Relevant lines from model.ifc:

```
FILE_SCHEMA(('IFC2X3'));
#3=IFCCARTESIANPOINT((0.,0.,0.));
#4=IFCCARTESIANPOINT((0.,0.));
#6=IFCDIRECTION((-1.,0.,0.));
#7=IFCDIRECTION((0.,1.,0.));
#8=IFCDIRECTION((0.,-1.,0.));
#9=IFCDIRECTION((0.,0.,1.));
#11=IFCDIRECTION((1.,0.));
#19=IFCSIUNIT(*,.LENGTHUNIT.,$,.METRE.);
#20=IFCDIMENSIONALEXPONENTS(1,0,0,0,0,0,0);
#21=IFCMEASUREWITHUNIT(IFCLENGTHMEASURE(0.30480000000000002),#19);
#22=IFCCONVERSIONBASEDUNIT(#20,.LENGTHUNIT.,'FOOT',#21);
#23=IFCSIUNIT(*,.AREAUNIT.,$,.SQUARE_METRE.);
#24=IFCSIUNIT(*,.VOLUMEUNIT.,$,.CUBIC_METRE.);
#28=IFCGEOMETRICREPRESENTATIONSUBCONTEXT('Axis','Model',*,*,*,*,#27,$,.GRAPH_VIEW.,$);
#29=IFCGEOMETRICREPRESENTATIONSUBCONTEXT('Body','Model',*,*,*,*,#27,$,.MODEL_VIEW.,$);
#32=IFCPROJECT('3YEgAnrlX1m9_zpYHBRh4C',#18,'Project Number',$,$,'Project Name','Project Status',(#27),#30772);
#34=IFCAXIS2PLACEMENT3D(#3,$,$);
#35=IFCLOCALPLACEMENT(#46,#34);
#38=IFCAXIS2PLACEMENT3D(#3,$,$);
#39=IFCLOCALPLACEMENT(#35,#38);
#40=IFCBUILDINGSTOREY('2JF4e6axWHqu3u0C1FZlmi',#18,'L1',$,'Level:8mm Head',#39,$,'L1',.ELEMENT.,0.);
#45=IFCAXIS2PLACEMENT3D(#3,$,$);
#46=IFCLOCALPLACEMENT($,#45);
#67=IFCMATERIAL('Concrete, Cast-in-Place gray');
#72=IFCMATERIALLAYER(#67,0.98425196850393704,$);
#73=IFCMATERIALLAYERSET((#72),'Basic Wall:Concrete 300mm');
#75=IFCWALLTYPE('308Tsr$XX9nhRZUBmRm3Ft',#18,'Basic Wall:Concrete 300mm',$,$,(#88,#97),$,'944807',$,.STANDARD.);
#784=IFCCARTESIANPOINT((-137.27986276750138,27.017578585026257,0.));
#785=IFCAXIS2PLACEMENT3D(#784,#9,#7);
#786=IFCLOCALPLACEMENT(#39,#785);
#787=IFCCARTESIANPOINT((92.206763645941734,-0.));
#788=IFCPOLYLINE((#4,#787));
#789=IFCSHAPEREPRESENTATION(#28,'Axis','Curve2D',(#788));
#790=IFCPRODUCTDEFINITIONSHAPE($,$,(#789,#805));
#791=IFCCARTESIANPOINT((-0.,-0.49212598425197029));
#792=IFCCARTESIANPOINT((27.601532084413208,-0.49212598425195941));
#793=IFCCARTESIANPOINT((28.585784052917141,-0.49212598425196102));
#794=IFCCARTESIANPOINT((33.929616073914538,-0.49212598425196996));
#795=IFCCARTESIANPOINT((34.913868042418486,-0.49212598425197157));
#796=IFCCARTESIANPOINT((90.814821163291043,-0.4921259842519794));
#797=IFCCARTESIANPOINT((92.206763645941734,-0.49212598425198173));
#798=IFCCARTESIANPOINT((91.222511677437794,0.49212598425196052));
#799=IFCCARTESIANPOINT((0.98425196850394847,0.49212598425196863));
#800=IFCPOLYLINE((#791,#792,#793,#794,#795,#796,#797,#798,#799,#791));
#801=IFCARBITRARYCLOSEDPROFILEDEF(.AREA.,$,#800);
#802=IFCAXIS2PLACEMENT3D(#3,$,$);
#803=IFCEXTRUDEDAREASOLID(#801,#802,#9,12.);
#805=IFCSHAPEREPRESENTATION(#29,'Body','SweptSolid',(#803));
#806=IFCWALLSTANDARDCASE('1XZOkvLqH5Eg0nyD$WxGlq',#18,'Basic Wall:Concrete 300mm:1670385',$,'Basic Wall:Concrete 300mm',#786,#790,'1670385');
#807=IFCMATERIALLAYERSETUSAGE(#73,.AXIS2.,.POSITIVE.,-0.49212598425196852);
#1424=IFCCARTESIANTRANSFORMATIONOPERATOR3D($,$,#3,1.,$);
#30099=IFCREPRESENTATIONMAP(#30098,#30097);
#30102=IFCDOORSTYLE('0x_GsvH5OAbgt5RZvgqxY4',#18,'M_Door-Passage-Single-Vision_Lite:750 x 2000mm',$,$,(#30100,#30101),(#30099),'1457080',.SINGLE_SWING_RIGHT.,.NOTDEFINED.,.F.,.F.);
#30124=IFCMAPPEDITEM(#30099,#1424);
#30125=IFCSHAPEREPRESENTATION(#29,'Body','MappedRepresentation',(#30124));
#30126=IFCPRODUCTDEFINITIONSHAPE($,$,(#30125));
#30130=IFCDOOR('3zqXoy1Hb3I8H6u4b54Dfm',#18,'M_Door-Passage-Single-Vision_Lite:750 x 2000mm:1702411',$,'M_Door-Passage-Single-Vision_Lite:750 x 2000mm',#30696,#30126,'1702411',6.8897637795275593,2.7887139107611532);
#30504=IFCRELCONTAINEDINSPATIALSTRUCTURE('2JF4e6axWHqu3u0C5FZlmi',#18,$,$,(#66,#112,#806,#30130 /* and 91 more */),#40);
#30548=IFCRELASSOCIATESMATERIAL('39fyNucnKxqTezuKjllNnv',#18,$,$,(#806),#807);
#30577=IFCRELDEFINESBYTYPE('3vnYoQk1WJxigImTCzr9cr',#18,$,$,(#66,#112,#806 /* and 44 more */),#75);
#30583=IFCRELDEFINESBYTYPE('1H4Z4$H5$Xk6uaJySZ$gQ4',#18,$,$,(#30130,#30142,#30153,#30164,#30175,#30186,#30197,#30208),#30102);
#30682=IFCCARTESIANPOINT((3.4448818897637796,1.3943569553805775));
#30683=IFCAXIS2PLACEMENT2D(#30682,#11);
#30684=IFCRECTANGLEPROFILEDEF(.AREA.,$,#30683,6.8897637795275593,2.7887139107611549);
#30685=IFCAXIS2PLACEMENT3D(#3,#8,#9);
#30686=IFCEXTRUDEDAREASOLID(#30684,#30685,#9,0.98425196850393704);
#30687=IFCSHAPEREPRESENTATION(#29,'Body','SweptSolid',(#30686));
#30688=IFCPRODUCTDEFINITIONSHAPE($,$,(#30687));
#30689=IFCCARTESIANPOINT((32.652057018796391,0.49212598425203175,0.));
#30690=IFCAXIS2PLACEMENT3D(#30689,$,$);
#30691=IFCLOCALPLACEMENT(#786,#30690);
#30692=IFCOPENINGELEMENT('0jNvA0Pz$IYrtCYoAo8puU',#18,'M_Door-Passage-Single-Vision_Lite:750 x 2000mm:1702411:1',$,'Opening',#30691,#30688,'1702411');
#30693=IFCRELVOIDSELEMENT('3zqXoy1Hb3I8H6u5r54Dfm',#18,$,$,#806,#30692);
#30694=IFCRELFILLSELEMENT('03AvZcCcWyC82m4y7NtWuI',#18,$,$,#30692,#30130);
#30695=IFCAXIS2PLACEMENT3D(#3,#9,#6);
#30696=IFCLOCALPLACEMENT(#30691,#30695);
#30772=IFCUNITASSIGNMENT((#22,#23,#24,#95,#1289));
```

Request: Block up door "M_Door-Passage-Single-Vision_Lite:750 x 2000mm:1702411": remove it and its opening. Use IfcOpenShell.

```python
import ifcopenshell
import ifcopenshell.api.feature
import ifcopenshell.api.root
import ifcopenshell.geom
import ifcopenshell.util.shape

model = ifcopenshell.open("model.ifc")
settings = ifcopenshell.geom.settings()


def volume(element):
    """Net volume in cubic metres, openings subtracted."""
    shape = ifcopenshell.geom.create_shape(settings, element)
    return ifcopenshell.util.shape.get_volume(shape.geometry)


door = model.by_guid("3zqXoy1Hb3I8H6u4b54Dfm")
opening = door.FillsVoids[0].RelatingOpeningElement
wall = opening.VoidsElements[0].RelatingBuildingElement
before = volume(wall)

ifcopenshell.api.root.remove_product(model, product=door)
ifcopenshell.api.feature.remove_feature(model, feature=opening)

after = volume(wall)

print(f"wall volume {before:.3f} -> {after:.3f} m3")

model.write("model_rev.ifc")
```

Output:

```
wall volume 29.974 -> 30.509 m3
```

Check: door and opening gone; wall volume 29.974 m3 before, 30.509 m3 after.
